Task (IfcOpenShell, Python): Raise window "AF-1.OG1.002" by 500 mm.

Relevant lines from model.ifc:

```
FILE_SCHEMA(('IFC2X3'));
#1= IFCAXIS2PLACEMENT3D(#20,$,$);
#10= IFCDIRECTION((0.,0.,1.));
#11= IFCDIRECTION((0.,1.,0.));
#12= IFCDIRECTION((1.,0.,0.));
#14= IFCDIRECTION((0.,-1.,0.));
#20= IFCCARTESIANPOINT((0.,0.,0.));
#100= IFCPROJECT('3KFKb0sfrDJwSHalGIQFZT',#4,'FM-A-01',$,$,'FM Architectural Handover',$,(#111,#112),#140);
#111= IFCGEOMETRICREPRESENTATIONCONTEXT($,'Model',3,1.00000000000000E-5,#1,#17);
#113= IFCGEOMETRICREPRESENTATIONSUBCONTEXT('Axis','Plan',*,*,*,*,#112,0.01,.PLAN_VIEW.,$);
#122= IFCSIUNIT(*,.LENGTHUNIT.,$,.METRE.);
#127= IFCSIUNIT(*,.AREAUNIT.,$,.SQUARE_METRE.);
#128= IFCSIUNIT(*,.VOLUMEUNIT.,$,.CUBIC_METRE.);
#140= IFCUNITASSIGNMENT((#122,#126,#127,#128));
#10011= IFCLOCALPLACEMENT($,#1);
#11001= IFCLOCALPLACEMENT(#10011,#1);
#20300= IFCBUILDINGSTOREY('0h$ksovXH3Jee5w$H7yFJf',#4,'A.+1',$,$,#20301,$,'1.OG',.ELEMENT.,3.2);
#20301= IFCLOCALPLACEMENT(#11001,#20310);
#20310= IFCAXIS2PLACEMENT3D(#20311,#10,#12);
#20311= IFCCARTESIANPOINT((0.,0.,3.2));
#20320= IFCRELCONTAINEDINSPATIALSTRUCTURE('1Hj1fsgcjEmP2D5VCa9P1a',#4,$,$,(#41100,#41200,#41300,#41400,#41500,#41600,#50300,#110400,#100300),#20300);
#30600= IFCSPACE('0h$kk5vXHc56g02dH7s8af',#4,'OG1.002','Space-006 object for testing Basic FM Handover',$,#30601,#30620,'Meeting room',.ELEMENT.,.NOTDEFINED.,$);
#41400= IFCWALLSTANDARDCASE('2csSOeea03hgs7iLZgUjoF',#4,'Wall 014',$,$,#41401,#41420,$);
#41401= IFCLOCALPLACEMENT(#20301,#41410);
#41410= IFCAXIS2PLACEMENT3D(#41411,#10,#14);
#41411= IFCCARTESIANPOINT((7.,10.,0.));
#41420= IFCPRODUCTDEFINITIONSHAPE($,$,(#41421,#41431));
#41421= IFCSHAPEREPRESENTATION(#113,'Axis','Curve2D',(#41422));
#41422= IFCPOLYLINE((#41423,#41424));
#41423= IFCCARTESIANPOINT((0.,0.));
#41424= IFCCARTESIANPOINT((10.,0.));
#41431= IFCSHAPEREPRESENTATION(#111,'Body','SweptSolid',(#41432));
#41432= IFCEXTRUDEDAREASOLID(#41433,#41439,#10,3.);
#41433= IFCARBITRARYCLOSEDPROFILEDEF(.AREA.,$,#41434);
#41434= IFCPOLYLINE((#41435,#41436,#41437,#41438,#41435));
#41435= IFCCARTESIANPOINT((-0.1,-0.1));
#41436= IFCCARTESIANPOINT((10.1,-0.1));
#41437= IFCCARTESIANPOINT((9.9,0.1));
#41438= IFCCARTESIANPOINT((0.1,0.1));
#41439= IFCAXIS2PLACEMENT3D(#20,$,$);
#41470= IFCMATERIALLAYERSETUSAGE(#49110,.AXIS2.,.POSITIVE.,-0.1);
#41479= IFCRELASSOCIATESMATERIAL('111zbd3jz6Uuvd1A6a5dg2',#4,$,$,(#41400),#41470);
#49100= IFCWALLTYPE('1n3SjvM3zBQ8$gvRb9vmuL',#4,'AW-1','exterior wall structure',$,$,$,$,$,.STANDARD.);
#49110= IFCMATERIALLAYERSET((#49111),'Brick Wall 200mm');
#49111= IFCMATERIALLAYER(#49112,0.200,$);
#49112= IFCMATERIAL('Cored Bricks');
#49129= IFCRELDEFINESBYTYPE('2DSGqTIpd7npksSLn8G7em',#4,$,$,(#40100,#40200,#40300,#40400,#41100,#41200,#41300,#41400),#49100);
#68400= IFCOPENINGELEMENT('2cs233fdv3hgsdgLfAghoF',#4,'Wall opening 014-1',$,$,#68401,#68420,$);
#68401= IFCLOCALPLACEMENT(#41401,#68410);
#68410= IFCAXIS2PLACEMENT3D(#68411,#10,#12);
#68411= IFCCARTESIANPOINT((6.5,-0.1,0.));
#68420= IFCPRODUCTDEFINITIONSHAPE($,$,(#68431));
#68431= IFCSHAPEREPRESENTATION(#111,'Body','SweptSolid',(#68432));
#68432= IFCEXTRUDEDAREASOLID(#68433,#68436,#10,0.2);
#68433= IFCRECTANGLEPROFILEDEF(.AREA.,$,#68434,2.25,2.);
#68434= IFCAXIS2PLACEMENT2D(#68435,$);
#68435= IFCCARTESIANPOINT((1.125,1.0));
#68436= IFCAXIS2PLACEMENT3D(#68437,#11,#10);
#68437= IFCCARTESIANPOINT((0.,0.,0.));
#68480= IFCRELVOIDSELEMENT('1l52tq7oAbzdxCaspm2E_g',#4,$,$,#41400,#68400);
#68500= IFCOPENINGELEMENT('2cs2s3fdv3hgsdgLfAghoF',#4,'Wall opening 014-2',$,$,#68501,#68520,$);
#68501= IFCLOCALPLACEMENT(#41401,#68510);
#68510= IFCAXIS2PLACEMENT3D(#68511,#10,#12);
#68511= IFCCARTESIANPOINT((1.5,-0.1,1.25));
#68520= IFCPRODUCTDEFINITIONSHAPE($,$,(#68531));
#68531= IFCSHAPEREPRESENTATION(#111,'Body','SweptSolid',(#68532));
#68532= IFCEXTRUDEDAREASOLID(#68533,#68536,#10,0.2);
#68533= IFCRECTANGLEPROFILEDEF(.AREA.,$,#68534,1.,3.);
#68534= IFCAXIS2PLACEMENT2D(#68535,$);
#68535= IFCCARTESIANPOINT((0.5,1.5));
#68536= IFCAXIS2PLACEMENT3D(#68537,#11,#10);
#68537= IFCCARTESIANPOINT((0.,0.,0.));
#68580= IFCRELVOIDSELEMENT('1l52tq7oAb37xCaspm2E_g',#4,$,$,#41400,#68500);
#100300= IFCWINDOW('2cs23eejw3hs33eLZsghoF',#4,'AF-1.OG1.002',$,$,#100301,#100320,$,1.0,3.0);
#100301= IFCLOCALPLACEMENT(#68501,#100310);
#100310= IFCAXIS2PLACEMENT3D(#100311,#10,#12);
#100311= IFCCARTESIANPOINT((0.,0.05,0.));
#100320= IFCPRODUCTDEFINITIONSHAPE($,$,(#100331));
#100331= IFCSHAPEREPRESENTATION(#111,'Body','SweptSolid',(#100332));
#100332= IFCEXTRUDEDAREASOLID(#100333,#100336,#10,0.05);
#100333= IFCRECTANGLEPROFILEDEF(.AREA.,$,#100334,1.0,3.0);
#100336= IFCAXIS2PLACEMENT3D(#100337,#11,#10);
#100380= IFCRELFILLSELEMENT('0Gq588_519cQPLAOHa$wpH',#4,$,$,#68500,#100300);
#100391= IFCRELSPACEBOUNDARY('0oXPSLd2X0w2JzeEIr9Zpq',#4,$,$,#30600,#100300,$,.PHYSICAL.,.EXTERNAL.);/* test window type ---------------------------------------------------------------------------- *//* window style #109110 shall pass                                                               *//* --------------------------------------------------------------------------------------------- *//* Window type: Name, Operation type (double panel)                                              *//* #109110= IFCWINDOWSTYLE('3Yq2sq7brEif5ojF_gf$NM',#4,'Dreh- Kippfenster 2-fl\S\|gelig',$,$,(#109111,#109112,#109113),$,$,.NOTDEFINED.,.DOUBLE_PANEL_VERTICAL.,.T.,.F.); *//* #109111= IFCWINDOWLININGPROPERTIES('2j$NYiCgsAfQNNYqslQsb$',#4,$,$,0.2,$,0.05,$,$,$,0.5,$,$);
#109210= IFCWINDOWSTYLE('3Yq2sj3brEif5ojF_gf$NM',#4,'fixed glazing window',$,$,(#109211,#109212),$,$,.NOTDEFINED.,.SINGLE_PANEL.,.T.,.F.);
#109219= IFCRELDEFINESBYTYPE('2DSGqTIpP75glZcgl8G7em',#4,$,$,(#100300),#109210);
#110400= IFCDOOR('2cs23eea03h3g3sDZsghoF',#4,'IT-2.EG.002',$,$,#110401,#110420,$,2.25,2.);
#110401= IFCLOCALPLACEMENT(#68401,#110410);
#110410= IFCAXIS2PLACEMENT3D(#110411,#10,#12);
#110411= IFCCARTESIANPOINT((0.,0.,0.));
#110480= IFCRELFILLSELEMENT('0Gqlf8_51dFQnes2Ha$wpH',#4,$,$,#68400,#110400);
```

```python
import numpy as np
import ifcopenshell
import ifcopenshell.api.geometry
import ifcopenshell.util.placement
import ifcopenshell.util.unit

model = ifcopenshell.open("model.ifc")
unit_scale = ifcopenshell.util.unit.calculate_unit_scale(model)

window = model.by_id(100300)
opening = window.FillsVoids[0].RelatingOpeningElement
dz = 0.5

shift = np.array([0.0, 0.0, dz])
# The window is placed relative to its opening, so it follows when the opening moves.
matrix = ifcopenshell.util.placement.get_local_placement(opening.ObjectPlacement)
matrix[:3, 3] += shift
ifcopenshell.api.geometry.edit_object_placement(
    model, product=opening, matrix=matrix, is_si=False, should_transform_children=True
)

print(f"moved by {dz * unit_scale:+.3f} m")

model.write("model_v2.ifc")
```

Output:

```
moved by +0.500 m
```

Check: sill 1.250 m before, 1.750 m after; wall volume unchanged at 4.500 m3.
